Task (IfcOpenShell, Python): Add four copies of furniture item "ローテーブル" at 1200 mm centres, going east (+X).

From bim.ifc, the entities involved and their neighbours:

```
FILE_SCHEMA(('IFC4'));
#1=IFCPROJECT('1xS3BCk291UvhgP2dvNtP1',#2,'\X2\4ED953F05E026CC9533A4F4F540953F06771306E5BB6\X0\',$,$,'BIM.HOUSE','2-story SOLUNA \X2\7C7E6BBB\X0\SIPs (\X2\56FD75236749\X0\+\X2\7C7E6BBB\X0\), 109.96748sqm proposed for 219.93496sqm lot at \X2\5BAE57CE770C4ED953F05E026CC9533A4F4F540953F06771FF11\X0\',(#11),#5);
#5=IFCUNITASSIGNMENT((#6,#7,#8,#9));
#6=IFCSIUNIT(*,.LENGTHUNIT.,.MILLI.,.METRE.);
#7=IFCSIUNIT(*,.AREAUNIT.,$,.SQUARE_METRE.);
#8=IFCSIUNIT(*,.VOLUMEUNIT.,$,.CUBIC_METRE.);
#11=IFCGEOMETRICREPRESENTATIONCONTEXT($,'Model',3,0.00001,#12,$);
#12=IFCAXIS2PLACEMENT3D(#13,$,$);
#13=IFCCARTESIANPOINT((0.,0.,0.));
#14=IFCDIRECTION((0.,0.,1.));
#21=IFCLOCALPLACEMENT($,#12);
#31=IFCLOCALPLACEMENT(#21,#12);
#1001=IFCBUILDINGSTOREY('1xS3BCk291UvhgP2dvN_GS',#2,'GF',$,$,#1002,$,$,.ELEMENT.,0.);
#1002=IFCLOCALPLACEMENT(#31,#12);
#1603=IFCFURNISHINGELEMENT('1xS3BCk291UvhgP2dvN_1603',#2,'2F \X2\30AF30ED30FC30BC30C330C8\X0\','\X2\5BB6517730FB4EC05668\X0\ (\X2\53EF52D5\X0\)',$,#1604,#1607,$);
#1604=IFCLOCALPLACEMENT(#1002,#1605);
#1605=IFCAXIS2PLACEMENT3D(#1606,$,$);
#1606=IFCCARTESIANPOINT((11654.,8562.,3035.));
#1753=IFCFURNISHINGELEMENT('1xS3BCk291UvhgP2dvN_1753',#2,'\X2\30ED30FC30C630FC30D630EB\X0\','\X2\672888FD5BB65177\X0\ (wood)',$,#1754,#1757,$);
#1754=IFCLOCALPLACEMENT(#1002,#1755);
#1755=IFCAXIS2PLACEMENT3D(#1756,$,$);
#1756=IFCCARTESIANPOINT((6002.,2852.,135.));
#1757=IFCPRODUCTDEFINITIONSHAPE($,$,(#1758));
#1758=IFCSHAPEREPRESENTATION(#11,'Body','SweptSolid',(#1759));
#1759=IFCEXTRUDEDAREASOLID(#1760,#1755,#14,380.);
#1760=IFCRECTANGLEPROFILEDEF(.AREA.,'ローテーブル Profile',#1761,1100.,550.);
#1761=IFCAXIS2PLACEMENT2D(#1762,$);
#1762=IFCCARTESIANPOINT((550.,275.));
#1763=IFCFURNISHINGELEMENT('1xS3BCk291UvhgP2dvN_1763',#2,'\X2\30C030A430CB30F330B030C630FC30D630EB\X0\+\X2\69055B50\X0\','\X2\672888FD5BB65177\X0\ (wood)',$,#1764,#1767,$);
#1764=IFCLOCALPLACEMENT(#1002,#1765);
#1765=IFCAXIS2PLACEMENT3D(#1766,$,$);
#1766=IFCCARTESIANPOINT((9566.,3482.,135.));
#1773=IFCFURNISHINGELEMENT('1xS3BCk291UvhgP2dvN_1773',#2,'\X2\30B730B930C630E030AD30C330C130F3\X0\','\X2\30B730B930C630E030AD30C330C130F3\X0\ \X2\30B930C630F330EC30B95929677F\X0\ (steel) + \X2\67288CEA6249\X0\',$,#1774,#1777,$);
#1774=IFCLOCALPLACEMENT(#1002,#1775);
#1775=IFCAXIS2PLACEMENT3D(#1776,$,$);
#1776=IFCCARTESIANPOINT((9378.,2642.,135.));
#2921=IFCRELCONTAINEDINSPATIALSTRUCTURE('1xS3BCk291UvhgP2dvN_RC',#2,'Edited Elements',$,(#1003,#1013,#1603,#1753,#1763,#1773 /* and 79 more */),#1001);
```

```python
import numpy as np
import ifcopenshell
import ifcopenshell.api.geometry
import ifcopenshell.api.root
import ifcopenshell.util.element
import ifcopenshell.util.placement

model = ifcopenshell.open("bim.ifc")


def reuse_history(source, copy):
    """copy_class also copies each property set's owner history, people and application; keep the originals."""
    for rel in copy.IsDefinedBy:
        if rel.is_a("IfcRelDefinesByProperties") and (history := rel.RelatingPropertyDefinition.OwnerHistory):
            rel.RelatingPropertyDefinition.OwnerHistory = source.OwnerHistory
            ifcopenshell.util.element.remove_deep2(model, history)


source = model.by_id(1753)
base = ifcopenshell.util.placement.get_local_placement(source.ObjectPlacement)
step = np.array([1.0, 0.0, 0.0]) * 1200.0

for i in range(1, 5):
    copy = ifcopenshell.api.root.copy_class(model, product=source)
    copy.Representation = ifcopenshell.util.element.copy_deep(
        model, source.Representation, exclude=["IfcGeometricRepresentationContext", "IfcRepresentationMap"]
    )
    reuse_history(source, copy)
    matrix = base.copy()
    matrix[:3, 3] += i * step
    print("added at", matrix[:3, 3].round(3) + 0.0)
    ifcopenshell.api.geometry.edit_object_placement(model, product=copy, matrix=matrix, is_si=False)

model.write("bim_rev.ifc")
```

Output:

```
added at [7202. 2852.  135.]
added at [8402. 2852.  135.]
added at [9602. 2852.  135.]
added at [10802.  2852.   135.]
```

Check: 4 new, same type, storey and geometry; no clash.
